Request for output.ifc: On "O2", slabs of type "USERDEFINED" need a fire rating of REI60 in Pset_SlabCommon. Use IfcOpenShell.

First a look at what the model holds.

```python
import ifcopenshell
import ifcopenshell.util.element

model = ifcopenshell.open("output.ifc")
print(model.schema)
storey = next(s for s in model.by_type("IfcBuildingStorey") if s.Name == "O2")
slabs = [e for e in ifcopenshell.util.element.get_decomposition(storey) if e.is_a("IfcSlab")]
seen = {}
for e in slabs:
    element_type = ifcopenshell.util.element.get_type(e)
    key = (element_type.Name if element_type != e and element_type else None, ifcopenshell.util.element.get_pset(e, "Pset_SlabCommon", "FireRating"))
    seen[key] = seen.get(key, 0) + 1
for (name, value), count in sorted(seen.items(), key=str):
    print(count, "x", name, "|", value)
```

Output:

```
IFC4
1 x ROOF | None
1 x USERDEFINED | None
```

```python
import ifcopenshell
import ifcopenshell.api.pset
import ifcopenshell.util.element

model = ifcopenshell.open("output.ifc")

storey = next(s for s in model.by_type("IfcBuildingStorey") if s.Name == "O2")
slabs = [e for e in ifcopenshell.util.element.get_decomposition(storey) if e.is_a("IfcSlab")]

count = 0
for e in slabs:
    element_type = ifcopenshell.util.element.get_type(e)
    if element_type in (None, e) or element_type.Name != "USERDEFINED":
        continue
    # add_pset returns the element's existing set when there is one.
    pset = ifcopenshell.api.pset.add_pset(model, product=e, name="Pset_SlabCommon")
    ifcopenshell.api.pset.edit_pset(model, pset=pset, properties={"FireRating": "REI60"})
    count += 1

print(count, "slabs updated")

model.write("output_edited.ifc")
```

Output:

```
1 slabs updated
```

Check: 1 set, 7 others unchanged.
